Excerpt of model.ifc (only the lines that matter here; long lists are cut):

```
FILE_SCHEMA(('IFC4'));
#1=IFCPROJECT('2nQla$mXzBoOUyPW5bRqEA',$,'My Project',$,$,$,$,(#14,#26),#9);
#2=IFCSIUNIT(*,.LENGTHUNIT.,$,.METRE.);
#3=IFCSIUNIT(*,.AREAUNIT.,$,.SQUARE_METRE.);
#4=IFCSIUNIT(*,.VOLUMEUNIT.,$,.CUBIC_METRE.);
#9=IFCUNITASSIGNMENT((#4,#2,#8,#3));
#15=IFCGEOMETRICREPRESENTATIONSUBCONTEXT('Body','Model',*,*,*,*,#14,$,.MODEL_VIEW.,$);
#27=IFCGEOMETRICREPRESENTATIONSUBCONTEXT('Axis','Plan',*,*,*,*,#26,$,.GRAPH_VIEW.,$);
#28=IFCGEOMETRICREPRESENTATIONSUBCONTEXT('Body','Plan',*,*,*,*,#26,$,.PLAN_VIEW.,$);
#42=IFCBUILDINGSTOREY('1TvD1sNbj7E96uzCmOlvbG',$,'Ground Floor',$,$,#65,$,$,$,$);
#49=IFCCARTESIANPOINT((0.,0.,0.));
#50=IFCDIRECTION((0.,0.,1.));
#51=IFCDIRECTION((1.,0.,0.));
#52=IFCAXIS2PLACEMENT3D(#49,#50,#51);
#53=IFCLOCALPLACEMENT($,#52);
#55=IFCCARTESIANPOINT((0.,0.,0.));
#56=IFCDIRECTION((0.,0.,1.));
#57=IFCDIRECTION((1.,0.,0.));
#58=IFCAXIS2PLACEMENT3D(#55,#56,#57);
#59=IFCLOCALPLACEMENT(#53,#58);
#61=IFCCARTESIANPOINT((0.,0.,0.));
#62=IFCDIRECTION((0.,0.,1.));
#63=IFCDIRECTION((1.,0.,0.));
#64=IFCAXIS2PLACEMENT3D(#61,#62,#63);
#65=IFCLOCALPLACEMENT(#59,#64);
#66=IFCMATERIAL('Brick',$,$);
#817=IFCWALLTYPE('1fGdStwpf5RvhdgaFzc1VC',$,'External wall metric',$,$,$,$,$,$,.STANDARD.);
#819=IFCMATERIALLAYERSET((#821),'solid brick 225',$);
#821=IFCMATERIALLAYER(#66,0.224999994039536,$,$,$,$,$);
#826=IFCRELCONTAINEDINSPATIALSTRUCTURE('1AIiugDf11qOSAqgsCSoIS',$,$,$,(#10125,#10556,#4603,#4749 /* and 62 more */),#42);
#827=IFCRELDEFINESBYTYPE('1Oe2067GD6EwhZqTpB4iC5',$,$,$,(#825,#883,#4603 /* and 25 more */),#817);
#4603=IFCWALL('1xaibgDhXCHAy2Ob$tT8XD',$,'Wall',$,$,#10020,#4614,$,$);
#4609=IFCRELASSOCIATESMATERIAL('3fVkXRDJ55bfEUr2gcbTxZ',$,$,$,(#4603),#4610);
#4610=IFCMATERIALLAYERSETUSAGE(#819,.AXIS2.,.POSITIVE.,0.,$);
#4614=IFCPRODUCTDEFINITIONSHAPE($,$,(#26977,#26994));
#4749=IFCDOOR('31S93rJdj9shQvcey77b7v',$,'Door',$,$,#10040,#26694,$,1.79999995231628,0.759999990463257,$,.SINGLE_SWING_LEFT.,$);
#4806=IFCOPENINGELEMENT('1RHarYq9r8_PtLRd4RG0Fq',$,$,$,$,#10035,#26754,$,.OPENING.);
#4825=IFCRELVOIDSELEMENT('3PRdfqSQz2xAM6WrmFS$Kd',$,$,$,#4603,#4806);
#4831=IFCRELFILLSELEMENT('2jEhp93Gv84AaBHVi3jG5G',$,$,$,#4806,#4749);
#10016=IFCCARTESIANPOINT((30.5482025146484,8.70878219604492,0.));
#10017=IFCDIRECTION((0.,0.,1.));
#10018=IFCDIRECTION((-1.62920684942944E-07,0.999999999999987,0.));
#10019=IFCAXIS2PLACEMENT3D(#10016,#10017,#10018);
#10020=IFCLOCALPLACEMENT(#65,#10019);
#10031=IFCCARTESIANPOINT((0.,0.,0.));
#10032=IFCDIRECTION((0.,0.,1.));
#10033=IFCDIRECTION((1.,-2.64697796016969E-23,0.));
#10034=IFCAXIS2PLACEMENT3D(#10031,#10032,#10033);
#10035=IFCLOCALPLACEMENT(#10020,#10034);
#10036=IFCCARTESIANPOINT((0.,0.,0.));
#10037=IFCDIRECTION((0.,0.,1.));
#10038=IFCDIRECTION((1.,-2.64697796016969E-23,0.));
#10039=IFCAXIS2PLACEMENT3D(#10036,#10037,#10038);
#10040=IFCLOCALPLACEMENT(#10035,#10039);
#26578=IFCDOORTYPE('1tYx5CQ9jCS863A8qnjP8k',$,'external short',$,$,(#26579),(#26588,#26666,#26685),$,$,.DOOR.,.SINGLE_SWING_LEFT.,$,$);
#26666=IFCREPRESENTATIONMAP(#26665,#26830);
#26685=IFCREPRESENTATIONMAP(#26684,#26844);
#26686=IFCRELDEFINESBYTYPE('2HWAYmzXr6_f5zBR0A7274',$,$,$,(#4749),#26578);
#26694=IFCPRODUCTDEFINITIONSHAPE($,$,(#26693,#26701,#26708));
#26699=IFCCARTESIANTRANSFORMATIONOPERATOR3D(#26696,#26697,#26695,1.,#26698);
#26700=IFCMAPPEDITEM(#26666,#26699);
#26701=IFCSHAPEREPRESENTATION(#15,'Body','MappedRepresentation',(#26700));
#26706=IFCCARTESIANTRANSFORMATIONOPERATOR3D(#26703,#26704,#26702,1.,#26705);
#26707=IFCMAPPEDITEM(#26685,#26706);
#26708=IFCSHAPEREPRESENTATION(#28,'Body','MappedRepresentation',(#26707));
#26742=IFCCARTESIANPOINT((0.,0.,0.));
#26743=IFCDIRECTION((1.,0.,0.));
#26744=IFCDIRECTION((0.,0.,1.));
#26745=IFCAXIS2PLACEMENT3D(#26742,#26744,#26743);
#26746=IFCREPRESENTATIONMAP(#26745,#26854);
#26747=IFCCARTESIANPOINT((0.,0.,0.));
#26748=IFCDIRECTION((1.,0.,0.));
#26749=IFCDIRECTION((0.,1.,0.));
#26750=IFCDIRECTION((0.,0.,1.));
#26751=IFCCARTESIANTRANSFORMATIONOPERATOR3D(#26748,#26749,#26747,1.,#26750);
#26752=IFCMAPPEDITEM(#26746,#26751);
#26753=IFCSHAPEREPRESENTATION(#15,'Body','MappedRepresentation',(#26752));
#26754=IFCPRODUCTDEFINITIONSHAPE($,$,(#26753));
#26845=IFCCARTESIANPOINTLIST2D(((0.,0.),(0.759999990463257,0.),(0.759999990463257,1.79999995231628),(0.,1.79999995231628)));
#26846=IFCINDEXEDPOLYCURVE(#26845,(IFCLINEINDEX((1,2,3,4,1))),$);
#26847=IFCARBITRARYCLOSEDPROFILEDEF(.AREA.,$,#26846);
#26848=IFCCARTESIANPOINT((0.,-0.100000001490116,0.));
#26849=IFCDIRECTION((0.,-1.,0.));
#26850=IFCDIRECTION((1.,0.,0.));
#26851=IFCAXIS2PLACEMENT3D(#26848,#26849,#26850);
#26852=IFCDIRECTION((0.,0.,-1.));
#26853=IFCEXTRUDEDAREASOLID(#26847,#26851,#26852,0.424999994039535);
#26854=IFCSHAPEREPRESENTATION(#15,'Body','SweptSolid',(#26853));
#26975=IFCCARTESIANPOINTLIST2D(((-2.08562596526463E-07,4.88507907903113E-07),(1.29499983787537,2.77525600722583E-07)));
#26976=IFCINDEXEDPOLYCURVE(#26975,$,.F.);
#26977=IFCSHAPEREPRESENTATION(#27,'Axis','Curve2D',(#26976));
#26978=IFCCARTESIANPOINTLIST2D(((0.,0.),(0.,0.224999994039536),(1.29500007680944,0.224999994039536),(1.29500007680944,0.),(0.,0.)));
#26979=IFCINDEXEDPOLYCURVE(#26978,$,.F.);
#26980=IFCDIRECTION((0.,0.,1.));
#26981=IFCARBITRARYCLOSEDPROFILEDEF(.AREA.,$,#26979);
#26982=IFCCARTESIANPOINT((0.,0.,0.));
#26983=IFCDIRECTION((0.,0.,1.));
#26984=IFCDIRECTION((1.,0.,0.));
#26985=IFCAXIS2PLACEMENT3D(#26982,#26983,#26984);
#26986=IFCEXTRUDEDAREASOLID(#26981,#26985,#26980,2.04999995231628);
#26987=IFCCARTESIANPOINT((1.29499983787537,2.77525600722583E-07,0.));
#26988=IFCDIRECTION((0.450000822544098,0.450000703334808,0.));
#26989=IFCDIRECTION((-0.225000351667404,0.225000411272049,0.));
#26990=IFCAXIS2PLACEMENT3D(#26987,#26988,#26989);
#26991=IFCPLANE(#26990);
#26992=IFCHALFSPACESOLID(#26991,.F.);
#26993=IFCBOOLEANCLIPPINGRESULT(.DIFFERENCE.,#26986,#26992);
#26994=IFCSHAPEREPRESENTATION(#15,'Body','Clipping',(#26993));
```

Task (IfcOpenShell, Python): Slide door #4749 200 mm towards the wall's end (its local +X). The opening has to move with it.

```python
import ifcopenshell
import ifcopenshell.api.geometry
import ifcopenshell.util.placement

model = ifcopenshell.open("model.ifc")

door = model.by_guid("31S93rJdj9shQvcey77b7v")
opening = door.FillsVoids[0].RelatingOpeningElement
wall = opening.VoidsElements[0].RelatingBuildingElement

wall_matrix = ifcopenshell.util.placement.get_local_placement(wall.ObjectPlacement)
shift = wall_matrix[:3, 0] * 0.2
before = ifcopenshell.util.placement.get_local_placement(door.ObjectPlacement)[:3, 3].copy()

# The door is placed relative to its opening, so it follows when the opening moves.
matrix = ifcopenshell.util.placement.get_local_placement(opening.ObjectPlacement)
matrix[:3, 3] += shift
ifcopenshell.api.geometry.edit_object_placement(
    model, product=opening, matrix=matrix, is_si=False, should_transform_children=True
)

after = ifcopenshell.util.placement.get_local_placement(door.ObjectPlacement)[:3, 3]
print("door moved by", (after - before).round(3) + 0.0)

model.write("model_rev.ifc")
```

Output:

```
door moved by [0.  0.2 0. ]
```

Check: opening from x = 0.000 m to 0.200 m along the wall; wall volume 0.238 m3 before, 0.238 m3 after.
